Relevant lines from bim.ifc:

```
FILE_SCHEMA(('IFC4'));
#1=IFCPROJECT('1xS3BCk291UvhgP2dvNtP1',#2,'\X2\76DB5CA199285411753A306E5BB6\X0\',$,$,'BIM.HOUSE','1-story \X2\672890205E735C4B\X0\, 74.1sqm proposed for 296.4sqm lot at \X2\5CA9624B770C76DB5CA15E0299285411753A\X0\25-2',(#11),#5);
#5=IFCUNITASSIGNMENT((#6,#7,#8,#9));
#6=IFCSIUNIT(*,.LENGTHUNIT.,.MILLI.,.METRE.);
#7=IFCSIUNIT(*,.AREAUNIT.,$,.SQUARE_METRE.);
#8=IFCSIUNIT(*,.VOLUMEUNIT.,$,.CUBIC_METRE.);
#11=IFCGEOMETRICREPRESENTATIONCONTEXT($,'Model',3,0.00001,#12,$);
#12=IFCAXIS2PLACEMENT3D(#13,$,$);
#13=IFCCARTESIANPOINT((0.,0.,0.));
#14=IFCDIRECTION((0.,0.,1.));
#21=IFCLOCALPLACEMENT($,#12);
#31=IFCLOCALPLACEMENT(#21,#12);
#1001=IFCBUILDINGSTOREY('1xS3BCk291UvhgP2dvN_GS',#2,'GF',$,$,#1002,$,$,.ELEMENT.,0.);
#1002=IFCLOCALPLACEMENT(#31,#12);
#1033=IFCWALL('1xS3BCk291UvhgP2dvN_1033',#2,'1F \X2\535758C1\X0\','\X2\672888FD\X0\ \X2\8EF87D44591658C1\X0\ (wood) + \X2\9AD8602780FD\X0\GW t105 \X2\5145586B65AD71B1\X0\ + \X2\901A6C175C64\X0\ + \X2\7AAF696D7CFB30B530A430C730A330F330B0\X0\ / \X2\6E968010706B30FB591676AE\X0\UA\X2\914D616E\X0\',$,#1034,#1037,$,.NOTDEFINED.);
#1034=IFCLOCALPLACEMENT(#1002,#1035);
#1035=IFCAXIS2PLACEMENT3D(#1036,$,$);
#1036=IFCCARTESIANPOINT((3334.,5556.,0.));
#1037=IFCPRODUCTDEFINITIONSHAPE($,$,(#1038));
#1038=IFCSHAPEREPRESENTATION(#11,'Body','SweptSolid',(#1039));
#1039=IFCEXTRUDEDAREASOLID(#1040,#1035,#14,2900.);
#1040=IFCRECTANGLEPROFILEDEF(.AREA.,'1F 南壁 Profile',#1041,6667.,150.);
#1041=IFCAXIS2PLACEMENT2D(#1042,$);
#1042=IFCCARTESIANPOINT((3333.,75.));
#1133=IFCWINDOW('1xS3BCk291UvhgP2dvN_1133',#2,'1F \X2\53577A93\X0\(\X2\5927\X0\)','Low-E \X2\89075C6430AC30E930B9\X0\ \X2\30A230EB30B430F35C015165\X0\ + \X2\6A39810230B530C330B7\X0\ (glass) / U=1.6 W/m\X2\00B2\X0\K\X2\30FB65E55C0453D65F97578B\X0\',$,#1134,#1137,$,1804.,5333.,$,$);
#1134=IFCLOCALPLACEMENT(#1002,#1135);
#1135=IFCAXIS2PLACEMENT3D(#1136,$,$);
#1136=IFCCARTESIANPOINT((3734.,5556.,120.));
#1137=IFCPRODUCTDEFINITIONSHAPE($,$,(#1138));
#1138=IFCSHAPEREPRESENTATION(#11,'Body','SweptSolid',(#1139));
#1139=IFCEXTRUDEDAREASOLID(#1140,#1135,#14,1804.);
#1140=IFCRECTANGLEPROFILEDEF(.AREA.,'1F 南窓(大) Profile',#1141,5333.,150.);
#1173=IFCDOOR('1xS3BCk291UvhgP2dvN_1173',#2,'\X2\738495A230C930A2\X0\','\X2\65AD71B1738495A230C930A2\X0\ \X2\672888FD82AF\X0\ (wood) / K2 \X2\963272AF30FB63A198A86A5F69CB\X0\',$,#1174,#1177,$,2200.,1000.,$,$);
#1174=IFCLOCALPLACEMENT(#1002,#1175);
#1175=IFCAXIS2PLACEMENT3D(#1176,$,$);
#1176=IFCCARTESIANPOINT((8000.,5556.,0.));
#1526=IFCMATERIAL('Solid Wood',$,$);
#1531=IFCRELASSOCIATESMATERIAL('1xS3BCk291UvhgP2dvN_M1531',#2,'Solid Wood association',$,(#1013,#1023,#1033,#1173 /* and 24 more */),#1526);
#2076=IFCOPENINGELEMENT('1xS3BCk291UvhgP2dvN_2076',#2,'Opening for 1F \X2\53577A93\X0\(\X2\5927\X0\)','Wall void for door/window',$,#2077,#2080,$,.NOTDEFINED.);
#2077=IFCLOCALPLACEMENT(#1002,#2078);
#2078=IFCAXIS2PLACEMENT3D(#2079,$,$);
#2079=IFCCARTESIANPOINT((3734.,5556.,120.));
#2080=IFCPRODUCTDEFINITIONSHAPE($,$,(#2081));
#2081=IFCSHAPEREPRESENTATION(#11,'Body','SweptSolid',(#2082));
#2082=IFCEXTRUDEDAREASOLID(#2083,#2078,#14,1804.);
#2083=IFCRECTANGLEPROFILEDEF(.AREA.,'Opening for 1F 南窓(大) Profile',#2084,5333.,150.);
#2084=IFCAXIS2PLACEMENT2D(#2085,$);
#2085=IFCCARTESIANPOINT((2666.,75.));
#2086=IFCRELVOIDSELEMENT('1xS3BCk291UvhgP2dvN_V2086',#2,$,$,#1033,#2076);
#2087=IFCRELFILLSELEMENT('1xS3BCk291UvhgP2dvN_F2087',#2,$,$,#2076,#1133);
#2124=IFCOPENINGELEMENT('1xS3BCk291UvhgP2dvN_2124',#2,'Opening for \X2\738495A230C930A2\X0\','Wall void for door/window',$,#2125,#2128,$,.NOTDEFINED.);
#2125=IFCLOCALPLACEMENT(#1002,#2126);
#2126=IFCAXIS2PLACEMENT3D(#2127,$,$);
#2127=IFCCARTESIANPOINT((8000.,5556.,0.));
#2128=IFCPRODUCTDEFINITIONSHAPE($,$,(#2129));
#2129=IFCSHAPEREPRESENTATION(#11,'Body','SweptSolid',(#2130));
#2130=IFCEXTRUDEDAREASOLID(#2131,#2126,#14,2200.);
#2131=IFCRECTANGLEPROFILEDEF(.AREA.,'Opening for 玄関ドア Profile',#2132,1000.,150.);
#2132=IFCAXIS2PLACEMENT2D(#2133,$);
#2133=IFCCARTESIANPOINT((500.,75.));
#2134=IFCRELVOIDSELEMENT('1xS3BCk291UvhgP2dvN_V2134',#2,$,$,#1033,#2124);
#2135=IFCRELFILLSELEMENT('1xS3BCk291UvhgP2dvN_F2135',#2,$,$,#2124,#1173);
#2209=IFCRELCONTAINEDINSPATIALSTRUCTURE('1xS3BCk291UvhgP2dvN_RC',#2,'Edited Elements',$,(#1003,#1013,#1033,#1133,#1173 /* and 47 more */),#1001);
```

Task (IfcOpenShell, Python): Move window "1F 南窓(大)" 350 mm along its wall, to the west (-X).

```python
import ifcopenshell
import ifcopenshell.api.geometry
import ifcopenshell.util.placement
import ifcopenshell.util.unit

model = ifcopenshell.open("bim.ifc")
unit_scale = ifcopenshell.util.unit.calculate_unit_scale(model)

window = model.by_id(1133)
opening = window.FillsVoids[0].RelatingOpeningElement
wall = opening.VoidsElements[0].RelatingBuildingElement

wall_matrix = ifcopenshell.util.placement.get_local_placement(wall.ObjectPlacement)
shift = wall_matrix[:3, 0] * -0.35 / unit_scale
before = ifcopenshell.util.placement.get_local_placement(window.ObjectPlacement)[:3, 3].copy()

# The window is not placed relative to its opening, so move both.
for product in (opening, window):
    matrix = ifcopenshell.util.placement.get_local_placement(product.ObjectPlacement)
    matrix[:3, 3] += shift
    ifcopenshell.api.geometry.edit_object_placement(model, product=product, matrix=matrix, is_si=False)

after = ifcopenshell.util.placement.get_local_placement(window.ObjectPlacement)[:3, 3]
print("window moved by", (after - before).round(3) + 0.0)

model.write("bim-out.ifc")
```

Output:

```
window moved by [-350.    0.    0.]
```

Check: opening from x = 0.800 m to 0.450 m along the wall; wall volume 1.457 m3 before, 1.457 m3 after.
